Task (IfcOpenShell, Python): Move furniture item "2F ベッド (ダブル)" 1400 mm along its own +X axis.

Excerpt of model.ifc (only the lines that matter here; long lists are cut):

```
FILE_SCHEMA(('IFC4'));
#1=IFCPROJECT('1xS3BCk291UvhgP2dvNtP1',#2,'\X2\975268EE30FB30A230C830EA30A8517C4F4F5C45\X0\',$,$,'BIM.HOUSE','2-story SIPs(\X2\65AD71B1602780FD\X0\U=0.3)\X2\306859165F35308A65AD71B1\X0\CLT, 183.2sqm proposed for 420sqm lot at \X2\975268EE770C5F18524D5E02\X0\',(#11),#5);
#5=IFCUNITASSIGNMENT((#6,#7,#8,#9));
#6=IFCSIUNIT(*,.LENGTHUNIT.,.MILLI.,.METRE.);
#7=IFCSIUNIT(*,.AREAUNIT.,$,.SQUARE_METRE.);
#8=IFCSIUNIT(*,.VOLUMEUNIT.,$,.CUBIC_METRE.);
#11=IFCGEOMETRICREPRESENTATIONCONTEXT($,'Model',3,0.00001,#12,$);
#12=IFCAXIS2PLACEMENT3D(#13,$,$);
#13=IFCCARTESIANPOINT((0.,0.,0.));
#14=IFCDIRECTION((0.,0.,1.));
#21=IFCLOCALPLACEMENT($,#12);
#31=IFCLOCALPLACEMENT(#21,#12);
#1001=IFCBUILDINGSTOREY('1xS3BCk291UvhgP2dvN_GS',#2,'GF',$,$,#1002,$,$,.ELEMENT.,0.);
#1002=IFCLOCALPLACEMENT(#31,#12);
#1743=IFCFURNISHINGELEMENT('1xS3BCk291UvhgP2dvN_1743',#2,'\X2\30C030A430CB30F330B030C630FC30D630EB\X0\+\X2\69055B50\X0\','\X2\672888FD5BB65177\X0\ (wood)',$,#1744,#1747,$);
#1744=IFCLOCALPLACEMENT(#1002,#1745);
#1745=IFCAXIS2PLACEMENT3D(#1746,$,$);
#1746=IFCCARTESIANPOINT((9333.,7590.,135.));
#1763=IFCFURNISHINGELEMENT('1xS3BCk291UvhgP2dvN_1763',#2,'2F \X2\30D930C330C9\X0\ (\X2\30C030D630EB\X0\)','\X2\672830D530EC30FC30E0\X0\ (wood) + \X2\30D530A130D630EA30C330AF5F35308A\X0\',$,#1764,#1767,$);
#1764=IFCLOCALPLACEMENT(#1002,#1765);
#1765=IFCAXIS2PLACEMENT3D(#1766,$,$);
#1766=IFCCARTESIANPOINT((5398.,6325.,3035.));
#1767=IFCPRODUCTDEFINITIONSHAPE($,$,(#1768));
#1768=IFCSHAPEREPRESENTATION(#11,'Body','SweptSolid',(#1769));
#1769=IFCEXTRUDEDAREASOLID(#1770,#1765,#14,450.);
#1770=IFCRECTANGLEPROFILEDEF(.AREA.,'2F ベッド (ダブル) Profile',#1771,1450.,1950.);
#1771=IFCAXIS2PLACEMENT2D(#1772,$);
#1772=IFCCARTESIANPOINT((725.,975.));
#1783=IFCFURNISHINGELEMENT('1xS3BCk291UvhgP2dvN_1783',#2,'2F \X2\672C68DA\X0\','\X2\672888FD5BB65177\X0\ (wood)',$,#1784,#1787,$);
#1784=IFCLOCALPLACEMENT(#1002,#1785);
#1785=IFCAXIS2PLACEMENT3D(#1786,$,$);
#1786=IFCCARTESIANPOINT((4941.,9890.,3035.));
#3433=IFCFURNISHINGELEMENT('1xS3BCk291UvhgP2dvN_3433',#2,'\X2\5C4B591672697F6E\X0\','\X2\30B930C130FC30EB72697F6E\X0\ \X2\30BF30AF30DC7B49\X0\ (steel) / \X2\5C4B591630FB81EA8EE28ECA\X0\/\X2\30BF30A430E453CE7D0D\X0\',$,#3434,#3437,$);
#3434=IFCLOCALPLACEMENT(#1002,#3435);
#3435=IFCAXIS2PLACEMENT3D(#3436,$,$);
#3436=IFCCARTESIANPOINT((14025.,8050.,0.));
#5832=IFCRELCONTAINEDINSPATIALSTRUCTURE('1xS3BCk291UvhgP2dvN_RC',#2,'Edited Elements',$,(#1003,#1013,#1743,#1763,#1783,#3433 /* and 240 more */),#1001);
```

```python
import ifcopenshell
import ifcopenshell.api.geometry
import ifcopenshell.util.placement

model = ifcopenshell.open("model.ifc")

item = model.by_guid("1xS3BCk291UvhgP2dvN_1763")
matrix = ifcopenshell.util.placement.get_local_placement(item.ObjectPlacement)
matrix[:3, 3] += matrix[:3, 0] * 1400.0
ifcopenshell.api.geometry.edit_object_placement(model, product=item, matrix=matrix, is_si=False)

print(ifcopenshell.util.placement.get_local_placement(item.ObjectPlacement).round(3) + 0.0)

model.write("model_rev.ifc")
```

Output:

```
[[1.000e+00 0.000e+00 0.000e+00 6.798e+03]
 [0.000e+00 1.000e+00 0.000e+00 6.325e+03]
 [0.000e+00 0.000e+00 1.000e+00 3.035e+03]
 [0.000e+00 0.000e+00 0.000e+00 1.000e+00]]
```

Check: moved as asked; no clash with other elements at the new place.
